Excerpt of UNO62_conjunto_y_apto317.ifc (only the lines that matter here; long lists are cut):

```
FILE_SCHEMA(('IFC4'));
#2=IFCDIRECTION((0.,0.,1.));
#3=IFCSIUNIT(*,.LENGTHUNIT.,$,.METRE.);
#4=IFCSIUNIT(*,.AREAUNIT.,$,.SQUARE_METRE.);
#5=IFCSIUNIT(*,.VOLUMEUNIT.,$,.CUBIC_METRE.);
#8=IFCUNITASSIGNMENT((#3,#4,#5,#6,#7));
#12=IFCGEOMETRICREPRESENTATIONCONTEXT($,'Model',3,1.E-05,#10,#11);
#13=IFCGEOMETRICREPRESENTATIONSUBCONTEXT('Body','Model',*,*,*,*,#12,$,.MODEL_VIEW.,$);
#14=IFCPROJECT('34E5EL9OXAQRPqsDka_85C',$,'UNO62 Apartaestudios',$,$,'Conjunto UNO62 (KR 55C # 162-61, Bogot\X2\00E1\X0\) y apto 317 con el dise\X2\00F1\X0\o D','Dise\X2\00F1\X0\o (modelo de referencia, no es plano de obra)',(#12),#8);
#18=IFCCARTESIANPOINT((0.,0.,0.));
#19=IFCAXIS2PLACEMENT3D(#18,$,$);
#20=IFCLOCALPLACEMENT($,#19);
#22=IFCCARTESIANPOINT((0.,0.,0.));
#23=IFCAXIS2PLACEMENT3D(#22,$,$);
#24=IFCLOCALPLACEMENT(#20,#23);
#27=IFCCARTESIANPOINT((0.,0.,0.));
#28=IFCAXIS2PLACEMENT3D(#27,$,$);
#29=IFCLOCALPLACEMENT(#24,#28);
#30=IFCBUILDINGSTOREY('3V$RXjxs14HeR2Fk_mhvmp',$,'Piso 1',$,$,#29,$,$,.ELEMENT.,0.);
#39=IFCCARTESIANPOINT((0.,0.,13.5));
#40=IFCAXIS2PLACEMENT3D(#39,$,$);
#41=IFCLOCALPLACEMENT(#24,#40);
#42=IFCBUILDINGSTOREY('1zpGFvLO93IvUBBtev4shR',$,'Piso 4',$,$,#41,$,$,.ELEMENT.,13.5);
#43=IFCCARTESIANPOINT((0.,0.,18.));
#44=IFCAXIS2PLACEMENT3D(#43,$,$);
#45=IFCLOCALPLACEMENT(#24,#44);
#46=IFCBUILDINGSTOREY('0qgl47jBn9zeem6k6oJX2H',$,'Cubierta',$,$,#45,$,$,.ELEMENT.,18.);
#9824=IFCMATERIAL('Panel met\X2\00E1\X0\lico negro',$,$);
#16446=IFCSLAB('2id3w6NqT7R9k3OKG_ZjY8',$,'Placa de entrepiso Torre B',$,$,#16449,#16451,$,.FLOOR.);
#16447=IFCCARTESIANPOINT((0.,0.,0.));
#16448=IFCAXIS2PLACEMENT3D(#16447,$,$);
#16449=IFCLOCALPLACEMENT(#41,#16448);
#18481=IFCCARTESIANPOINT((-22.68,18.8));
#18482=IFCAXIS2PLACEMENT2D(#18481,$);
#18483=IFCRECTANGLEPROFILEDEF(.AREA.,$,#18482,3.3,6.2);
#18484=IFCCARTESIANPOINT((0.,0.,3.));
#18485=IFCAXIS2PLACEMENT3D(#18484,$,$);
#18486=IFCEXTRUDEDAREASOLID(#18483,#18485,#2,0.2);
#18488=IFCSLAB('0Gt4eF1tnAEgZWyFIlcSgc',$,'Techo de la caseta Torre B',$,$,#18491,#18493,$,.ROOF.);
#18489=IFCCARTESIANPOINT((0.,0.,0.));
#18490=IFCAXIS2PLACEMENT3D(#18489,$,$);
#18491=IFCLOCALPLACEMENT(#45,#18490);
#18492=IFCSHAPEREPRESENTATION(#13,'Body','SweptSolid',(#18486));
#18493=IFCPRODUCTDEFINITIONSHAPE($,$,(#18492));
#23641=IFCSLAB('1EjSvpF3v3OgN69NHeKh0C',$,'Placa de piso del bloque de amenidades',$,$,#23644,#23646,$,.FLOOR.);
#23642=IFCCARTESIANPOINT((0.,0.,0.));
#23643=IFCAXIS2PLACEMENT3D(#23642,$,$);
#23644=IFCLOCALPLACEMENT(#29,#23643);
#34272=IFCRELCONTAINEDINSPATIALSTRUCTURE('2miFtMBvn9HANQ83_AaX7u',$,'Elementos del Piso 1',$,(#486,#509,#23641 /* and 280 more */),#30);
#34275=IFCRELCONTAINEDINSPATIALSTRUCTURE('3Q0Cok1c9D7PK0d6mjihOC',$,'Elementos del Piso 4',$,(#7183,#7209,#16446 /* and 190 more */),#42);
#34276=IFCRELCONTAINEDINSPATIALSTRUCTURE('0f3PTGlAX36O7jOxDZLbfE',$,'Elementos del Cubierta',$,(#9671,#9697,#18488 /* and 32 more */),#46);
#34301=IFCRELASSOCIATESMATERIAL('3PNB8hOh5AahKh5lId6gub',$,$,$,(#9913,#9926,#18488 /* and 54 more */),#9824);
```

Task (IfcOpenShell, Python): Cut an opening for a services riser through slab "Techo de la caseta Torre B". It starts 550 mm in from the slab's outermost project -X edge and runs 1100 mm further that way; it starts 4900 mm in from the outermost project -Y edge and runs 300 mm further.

```python
import numpy as np
import ifcopenshell
import ifcopenshell.api.feature
import ifcopenshell.api.geometry
import ifcopenshell.api.root
import ifcopenshell.geom
import ifcopenshell.util.placement
import ifcopenshell.util.representation
import ifcopenshell.util.shape
import ifcopenshell.util.unit

model = ifcopenshell.open("UNO62_conjunto_y_apto317.ifc")
unit_scale = ifcopenshell.util.unit.calculate_unit_scale(model)
settings = ifcopenshell.geom.settings()


def volume(element):
    """Net volume in cubic metres, openings subtracted."""
    shape = ifcopenshell.geom.create_shape(settings, element)
    return ifcopenshell.util.shape.get_volume(shape.geometry)


slab = model.by_guid("0Gt4eF1tnAEgZWyFIlcSgc")
before = volume(slab)

# Extent in the slab's own axes, in metres. The edges named are its -X and -Y sides.
slab_shape = ifcopenshell.geom.create_shape(settings, slab)
vertices = ifcopenshell.util.shape.get_vertices(slab_shape.geometry)
x_min, y_min, bottom = vertices.min(axis=0)
top = vertices[:, 2].max()

opening = ifcopenshell.api.root.create_entity(model, ifc_class="IfcOpeningElement", name="Services riser opening", predefined_type="OPENING")
context = ifcopenshell.util.representation.get_context(model, "Model", "Body", "MODEL_VIEW")
width, depth = 1.1, 0.3
outline = [(0.0, 0.0), (width, 0.0), (width, depth), (0.0, depth), (0.0, 0.0)]
# Overshoot both faces by 50 mm so the cut is clean.
shape = ifcopenshell.api.geometry.add_slab_representation(
    model, context=context, depth=top - bottom + 0.1, polyline=outline
)
ifcopenshell.api.geometry.assign_representation(model, product=opening, representation=shape)

matrix = ifcopenshell.util.placement.get_local_placement(slab.ObjectPlacement)
matrix[:, 3] = matrix @ np.append(np.array([x_min + 0.55, y_min + 4.9, bottom - 0.05]) / unit_scale, 1.0)
ifcopenshell.api.geometry.edit_object_placement(model, product=opening, matrix=matrix, is_si=False)
ifcopenshell.api.feature.add_feature(model, feature=opening, element=slab)

after = volume(slab)

print(f"slab volume {before:.3f} -> {after:.3f} m3")

model.write("UNO62_conjunto_y_apto317_edited.ifc")
```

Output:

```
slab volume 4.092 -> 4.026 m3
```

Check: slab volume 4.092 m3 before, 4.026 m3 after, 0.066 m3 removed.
